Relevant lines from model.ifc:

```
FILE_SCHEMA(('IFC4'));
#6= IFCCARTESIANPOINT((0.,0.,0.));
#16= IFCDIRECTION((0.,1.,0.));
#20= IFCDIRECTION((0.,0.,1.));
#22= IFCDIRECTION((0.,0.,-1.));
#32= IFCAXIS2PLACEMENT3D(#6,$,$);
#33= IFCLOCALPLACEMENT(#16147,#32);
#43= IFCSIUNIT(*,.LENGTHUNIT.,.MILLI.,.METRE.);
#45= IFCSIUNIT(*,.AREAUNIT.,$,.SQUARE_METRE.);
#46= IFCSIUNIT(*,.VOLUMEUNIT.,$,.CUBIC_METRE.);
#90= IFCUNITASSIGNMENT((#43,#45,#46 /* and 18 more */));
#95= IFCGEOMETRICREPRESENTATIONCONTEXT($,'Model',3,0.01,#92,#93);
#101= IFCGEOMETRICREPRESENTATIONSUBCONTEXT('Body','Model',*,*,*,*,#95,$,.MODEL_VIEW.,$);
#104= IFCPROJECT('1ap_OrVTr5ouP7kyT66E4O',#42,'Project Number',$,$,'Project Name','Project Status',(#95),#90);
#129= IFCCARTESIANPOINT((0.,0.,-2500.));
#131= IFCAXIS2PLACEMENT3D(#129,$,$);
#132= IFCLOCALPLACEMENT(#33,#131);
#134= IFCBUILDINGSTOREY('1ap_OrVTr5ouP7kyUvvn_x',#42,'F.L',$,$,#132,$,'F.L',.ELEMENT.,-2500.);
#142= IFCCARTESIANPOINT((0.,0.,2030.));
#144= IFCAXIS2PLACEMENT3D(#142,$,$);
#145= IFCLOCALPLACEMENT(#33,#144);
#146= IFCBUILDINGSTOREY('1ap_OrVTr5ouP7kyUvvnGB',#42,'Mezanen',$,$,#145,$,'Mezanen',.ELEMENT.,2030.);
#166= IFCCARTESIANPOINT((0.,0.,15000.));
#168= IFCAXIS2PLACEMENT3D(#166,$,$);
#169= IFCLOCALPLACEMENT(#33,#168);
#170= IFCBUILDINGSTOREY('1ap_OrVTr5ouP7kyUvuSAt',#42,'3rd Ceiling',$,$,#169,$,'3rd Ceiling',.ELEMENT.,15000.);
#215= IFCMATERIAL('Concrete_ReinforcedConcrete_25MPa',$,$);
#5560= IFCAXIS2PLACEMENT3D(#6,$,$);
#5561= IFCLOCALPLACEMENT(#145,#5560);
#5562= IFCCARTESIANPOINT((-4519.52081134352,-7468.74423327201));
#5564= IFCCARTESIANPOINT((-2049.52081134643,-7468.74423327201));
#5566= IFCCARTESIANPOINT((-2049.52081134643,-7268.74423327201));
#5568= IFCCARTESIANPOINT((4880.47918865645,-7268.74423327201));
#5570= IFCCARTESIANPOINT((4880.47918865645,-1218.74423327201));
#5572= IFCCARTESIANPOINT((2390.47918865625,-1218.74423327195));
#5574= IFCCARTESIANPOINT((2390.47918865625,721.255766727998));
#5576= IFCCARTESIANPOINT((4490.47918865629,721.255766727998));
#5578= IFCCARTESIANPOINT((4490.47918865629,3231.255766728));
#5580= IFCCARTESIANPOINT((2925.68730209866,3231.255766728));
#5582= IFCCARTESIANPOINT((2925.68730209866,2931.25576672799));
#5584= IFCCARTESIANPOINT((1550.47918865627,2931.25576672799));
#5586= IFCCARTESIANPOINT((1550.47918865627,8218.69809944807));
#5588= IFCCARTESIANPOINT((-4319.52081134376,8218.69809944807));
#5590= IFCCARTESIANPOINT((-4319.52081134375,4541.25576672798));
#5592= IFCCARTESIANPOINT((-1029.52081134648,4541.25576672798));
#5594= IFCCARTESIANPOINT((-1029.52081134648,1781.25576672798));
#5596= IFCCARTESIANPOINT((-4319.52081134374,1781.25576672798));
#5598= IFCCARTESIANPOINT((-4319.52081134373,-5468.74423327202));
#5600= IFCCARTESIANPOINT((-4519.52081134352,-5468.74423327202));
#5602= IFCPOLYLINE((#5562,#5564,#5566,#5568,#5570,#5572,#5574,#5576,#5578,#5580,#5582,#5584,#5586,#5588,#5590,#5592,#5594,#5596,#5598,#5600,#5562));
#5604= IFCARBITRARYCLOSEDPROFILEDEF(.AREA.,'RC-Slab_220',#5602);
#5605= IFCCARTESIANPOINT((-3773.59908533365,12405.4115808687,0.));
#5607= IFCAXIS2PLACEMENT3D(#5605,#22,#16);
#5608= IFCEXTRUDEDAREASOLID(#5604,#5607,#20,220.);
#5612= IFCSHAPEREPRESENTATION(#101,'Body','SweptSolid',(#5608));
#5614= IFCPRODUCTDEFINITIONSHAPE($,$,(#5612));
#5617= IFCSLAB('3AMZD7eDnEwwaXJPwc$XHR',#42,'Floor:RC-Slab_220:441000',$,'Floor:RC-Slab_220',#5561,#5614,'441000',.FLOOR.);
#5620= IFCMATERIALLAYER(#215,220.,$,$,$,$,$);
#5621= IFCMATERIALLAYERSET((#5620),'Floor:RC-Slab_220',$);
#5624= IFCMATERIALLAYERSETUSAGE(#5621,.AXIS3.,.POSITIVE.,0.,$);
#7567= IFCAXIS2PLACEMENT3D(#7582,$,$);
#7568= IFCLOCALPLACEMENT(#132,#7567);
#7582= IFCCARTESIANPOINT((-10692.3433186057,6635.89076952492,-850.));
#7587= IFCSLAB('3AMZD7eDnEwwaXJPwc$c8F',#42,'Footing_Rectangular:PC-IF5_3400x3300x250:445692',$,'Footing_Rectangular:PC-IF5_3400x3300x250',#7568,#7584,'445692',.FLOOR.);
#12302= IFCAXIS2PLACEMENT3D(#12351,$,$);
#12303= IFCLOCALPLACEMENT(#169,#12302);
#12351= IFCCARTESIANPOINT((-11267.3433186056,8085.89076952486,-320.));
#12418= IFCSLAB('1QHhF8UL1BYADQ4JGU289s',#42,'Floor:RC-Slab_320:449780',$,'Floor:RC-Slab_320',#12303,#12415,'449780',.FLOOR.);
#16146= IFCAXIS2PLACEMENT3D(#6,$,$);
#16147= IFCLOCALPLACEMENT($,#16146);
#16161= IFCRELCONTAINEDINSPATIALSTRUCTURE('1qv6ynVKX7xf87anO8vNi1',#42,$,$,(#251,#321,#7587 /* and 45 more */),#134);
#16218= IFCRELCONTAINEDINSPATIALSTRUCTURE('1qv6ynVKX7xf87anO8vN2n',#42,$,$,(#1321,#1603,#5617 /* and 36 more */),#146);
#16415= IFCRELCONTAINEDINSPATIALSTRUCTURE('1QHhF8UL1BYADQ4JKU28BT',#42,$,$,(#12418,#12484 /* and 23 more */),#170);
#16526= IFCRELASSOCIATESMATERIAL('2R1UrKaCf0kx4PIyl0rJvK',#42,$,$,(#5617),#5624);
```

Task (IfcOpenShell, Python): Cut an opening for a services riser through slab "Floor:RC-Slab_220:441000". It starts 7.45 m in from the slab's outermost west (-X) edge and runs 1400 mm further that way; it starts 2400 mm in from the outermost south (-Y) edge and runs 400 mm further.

```python
import numpy as np
import ifcopenshell
import ifcopenshell.api.feature
import ifcopenshell.api.geometry
import ifcopenshell.api.root
import ifcopenshell.geom
import ifcopenshell.util.placement
import ifcopenshell.util.representation
import ifcopenshell.util.shape
import ifcopenshell.util.unit

model = ifcopenshell.open("model.ifc")
unit_scale = ifcopenshell.util.unit.calculate_unit_scale(model)
settings = ifcopenshell.geom.settings()


def volume(element):
    """Net volume in cubic metres, openings subtracted."""
    shape = ifcopenshell.geom.create_shape(settings, element)
    return ifcopenshell.util.shape.get_volume(shape.geometry)


slab = model.by_guid("3AMZD7eDnEwwaXJPwc$XHR")
before = volume(slab)

# Extent in the slab's own axes, in metres. The edges named are its -X and -Y sides.
slab_shape = ifcopenshell.geom.create_shape(settings, slab)
vertices = ifcopenshell.util.shape.get_vertices(slab_shape.geometry)
x_min, y_min, bottom = vertices.min(axis=0)
top = vertices[:, 2].max()

opening = ifcopenshell.api.root.create_entity(model, ifc_class="IfcOpeningElement", name="Services riser opening", predefined_type="OPENING")
context = ifcopenshell.util.representation.get_context(model, "Model", "Body", "MODEL_VIEW")
width, depth = 1.4, 0.4
outline = [(0.0, 0.0), (width, 0.0), (width, depth), (0.0, depth), (0.0, 0.0)]
# Overshoot both faces by 50 mm so the cut is clean.
shape = ifcopenshell.api.geometry.add_slab_representation(
    model, context=context, depth=top - bottom + 0.1, polyline=outline
)
ifcopenshell.api.geometry.assign_representation(model, product=opening, representation=shape)

matrix = ifcopenshell.util.placement.get_local_placement(slab.ObjectPlacement)
matrix[:, 3] = matrix @ np.append(np.array([x_min + 7.45, y_min + 2.4, bottom - 0.05]) / unit_scale, 1.0)
ifcopenshell.api.geometry.edit_object_placement(model, product=opening, matrix=matrix, is_si=False)
ifcopenshell.api.feature.add_feature(model, feature=opening, element=slab)

after = volume(slab)

print(f"slab volume {before:.3f} -> {after:.3f} m3")

model.write("model_updated.ifc")
```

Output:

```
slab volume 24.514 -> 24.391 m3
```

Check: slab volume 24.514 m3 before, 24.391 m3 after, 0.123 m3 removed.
